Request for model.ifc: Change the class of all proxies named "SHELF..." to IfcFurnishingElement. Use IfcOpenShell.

First a look at what the model holds.

```python
import re

import ifcopenshell

model = ifcopenshell.open("model.ifc")
print(model.schema)
seen = {}
for e in model.by_type("IfcBuildingElementProxy"):
    name = re.sub(r":\d+(:\d+)?$", "", e.Name or "")  # drop the element id that some exporters append
    seen[name] = seen.get(name, 0) + 1
for name, count in sorted(seen.items()):
    print(count, "x", name)
```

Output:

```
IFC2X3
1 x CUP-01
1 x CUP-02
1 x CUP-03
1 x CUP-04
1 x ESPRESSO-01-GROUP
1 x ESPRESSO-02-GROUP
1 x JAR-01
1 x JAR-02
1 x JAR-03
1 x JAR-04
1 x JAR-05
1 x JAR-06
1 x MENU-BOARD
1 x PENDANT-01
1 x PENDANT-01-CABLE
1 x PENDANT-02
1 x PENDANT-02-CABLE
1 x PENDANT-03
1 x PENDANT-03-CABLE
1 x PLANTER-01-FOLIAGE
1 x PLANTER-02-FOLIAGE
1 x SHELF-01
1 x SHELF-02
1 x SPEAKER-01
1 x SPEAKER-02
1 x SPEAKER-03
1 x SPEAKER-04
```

```python
import ifcopenshell
import ifcopenshell.api.root

model = ifcopenshell.open("model.ifc")

proxies = [e.id() for e in model.by_type("IfcBuildingElementProxy") if (e.Name or "").startswith("SHELF")]
for step_id in proxies:
    proxy = model.by_id(step_id)
    ifcopenshell.api.root.reassign_class(model, product=proxy, ifc_class="IfcFurnishingElement")

print(sum(model.by_id(i).is_a("IfcFurnishingElement") for i in proxies), "reclassified")

model.write("model-out.ifc")
```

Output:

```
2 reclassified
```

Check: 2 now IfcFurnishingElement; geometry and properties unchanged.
